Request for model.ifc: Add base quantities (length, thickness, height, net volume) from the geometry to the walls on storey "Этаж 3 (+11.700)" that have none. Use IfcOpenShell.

First a look at what the model holds.

```python
import ifcopenshell
import ifcopenshell.util.element
import ifcopenshell.util.unit

model = ifcopenshell.open("model.ifc")
print(model.schema)
for unit_type in ("LENGTHUNIT", "AREAUNIT", "VOLUMEUNIT"):
    print(unit_type, ifcopenshell.util.unit.calculate_unit_scale(model, unit_type))
storey = next(s for s in model.by_type("IfcBuildingStorey") if s.Name == "Этаж 3 (+11.700)")
walls = [e for e in ifcopenshell.util.element.get_decomposition(storey) if e.is_a("IfcWall")]
for e in sorted(walls, key=lambda e: e.id()):
    print(e.id(), e.is_a(), e.Name, list(ifcopenshell.util.element.get_psets(e, qtos_only=True)), sep=" | ")
```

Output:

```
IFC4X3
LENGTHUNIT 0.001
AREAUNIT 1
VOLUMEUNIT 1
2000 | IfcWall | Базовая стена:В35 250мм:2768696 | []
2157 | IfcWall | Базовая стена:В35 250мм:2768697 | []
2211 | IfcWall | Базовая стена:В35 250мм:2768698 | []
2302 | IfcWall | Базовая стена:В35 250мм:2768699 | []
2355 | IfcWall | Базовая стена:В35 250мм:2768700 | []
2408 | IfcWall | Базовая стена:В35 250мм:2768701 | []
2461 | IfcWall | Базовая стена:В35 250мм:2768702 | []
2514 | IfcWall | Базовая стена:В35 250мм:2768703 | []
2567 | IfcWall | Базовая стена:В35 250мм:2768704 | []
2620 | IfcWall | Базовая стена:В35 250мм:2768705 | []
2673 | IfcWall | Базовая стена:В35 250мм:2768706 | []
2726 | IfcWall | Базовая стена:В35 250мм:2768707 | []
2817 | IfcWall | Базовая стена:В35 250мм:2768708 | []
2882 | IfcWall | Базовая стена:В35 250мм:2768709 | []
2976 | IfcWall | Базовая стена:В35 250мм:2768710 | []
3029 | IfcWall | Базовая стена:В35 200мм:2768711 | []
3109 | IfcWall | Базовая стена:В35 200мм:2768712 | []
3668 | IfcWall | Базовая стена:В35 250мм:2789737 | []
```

```python
import ifcopenshell
import ifcopenshell.api.pset
import ifcopenshell.geom
import ifcopenshell.util.element
import ifcopenshell.util.shape
import ifcopenshell.util.unit

model = ifcopenshell.open("model.ifc")
unit_scale = ifcopenshell.util.unit.calculate_unit_scale(model)
volume_scale = ifcopenshell.util.unit.calculate_unit_scale(model, "VOLUMEUNIT")
settings = ifcopenshell.geom.settings()

storey = next(s for s in model.by_type("IfcBuildingStorey") if s.Name == "Этаж 3 (+11.700)")
walls = [e for e in ifcopenshell.util.element.get_decomposition(storey) if e.is_a("IfcWall")]

for e in sorted(walls, key=lambda e: e.id()):
    if ifcopenshell.util.element.get_psets(e, qtos_only=True, should_inherit=False):
        continue
    # Geometry comes back in metres, in the element's own axes.
    shape = ifcopenshell.geom.create_shape(settings, e)
    values = {
        "Length": ifcopenshell.util.shape.get_x(shape.geometry) / unit_scale,
        "Width": ifcopenshell.util.shape.get_y(shape.geometry) / unit_scale,
        "Height": ifcopenshell.util.shape.get_z(shape.geometry) / unit_scale,
        "NetVolume": ifcopenshell.util.shape.get_volume(shape.geometry) / volume_scale,
    }
    qto = ifcopenshell.api.pset.add_qto(model, product=e, name="Qto_WallBaseQuantities")
    ifcopenshell.api.pset.edit_qto(model, qto=qto, properties=values)
    print(e.id(), {k: round(v, 3) for k, v in values.items()})

model.write("model_edited.ifc")
```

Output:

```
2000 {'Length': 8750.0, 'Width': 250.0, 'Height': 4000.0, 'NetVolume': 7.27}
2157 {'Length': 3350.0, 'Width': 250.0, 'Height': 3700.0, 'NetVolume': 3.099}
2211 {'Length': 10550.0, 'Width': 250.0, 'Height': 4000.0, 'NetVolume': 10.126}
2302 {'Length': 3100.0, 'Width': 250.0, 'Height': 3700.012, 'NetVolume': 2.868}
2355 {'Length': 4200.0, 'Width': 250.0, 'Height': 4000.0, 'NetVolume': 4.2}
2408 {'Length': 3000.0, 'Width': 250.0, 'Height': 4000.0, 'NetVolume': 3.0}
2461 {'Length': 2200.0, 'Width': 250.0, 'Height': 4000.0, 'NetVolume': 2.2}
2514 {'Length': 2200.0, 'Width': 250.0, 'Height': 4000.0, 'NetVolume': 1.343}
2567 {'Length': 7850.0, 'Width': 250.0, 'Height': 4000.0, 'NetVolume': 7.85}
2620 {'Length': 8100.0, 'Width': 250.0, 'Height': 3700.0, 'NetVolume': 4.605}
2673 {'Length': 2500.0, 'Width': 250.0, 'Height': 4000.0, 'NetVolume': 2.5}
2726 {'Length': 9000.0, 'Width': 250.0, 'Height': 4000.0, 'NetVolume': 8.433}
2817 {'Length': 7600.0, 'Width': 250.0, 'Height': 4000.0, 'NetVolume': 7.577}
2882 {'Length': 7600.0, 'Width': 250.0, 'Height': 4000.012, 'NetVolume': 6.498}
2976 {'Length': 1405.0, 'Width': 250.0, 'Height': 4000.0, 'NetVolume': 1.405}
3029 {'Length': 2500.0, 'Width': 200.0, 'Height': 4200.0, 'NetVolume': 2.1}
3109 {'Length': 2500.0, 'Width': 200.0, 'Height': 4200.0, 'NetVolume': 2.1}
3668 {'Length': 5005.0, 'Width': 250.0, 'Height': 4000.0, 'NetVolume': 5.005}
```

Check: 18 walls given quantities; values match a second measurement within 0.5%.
